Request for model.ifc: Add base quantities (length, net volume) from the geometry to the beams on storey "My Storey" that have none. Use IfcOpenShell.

First a look at what the model holds.

```python
import ifcopenshell
import ifcopenshell.util.element
import ifcopenshell.util.unit

model = ifcopenshell.open("model.ifc")
print(model.schema)
for unit_type in ("LENGTHUNIT", "AREAUNIT", "VOLUMEUNIT"):
    print(unit_type, ifcopenshell.util.unit.calculate_unit_scale(model, unit_type))
storey = next(s for s in model.by_type("IfcBuildingStorey") if s.Name == "My Storey")
beams = [e for e in ifcopenshell.util.element.get_decomposition(storey) if e.is_a("IfcBeam")]
for e in sorted(beams, key=lambda e: e.id()):
    print(e.id(), e.is_a(), e.Name, list(ifcopenshell.util.element.get_psets(e, qtos_only=True)), sep=" | ")
```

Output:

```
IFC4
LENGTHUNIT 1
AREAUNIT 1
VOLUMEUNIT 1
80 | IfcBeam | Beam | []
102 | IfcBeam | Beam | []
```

```python
import ifcopenshell
import ifcopenshell.api.pset
import ifcopenshell.geom
import ifcopenshell.util.element
import ifcopenshell.util.shape
import ifcopenshell.util.unit

model = ifcopenshell.open("model.ifc")
unit_scale = ifcopenshell.util.unit.calculate_unit_scale(model)
volume_scale = ifcopenshell.util.unit.calculate_unit_scale(model, "VOLUMEUNIT")
settings = ifcopenshell.geom.settings()

storey = next(s for s in model.by_type("IfcBuildingStorey") if s.Name == "My Storey")
beams = [e for e in ifcopenshell.util.element.get_decomposition(storey) if e.is_a("IfcBeam")]

for e in sorted(beams, key=lambda e: e.id()):
    if ifcopenshell.util.element.get_psets(e, qtos_only=True, should_inherit=False):
        continue
    # Geometry comes back in metres, in the element's own axes.
    shape = ifcopenshell.geom.create_shape(settings, e)
    values = {
        "Length": ifcopenshell.util.shape.get_max_xyz(shape.geometry) / unit_scale,
        "NetVolume": ifcopenshell.util.shape.get_volume(shape.geometry) / volume_scale,
    }
    qto = ifcopenshell.api.pset.add_qto(model, product=e, name="Qto_BeamBaseQuantities")
    ifcopenshell.api.pset.edit_qto(model, qto=qto, properties=values)
    print(e.id(), {k: round(v, 3) for k, v in values.items()})

model.write("model_edited.ifc")
```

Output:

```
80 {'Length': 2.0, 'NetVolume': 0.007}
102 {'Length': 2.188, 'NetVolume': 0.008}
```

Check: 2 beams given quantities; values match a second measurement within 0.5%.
